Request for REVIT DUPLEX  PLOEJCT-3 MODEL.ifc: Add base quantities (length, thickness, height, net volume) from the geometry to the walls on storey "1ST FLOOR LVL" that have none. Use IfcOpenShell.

First a look at what the model holds.

```python
import ifcopenshell
import ifcopenshell.util.element
import ifcopenshell.util.unit

model = ifcopenshell.open("REVIT DUPLEX  PLOEJCT-3 MODEL.ifc")
print(model.schema)
for unit_type in ("LENGTHUNIT", "AREAUNIT", "VOLUMEUNIT"):
    print(unit_type, ifcopenshell.util.unit.calculate_unit_scale(model, unit_type))
storey = next(s for s in model.by_type("IfcBuildingStorey") if s.Name == "1ST FLOOR LVL")
walls = [e for e in ifcopenshell.util.element.get_decomposition(storey) if e.is_a("IfcWall")]
for e in sorted(walls, key=lambda e: e.id()):
    print(e.id(), e.is_a(), e.Name, list(ifcopenshell.util.element.get_psets(e, qtos_only=True)), sep=" | ")
```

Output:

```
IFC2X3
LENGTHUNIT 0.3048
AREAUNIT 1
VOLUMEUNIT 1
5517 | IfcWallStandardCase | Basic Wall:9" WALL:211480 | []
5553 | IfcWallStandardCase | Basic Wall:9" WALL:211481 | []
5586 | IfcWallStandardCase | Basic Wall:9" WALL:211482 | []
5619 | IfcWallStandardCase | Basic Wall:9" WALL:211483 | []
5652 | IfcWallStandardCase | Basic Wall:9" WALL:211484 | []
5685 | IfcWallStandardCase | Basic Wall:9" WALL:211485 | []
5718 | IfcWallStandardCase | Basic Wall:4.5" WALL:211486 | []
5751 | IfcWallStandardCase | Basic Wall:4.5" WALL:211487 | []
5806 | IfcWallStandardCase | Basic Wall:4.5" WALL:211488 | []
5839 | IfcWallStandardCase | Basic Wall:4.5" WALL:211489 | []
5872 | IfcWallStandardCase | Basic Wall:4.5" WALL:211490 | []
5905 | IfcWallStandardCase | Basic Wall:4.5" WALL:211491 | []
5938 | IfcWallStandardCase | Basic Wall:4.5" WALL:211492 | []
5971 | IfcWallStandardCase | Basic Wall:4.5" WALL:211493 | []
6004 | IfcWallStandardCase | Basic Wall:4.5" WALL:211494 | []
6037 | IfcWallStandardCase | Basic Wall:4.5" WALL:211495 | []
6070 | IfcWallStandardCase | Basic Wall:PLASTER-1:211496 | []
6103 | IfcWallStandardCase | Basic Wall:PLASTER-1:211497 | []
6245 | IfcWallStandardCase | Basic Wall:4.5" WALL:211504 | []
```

```python
import ifcopenshell
import ifcopenshell.api.pset
import ifcopenshell.geom
import ifcopenshell.util.element
import ifcopenshell.util.shape
import ifcopenshell.util.unit

model = ifcopenshell.open("REVIT DUPLEX  PLOEJCT-3 MODEL.ifc")
unit_scale = ifcopenshell.util.unit.calculate_unit_scale(model)
volume_scale = ifcopenshell.util.unit.calculate_unit_scale(model, "VOLUMEUNIT")
settings = ifcopenshell.geom.settings()

storey = next(s for s in model.by_type("IfcBuildingStorey") if s.Name == "1ST FLOOR LVL")
walls = [e for e in ifcopenshell.util.element.get_decomposition(storey) if e.is_a("IfcWall")]

for e in sorted(walls, key=lambda e: e.id()):
    if ifcopenshell.util.element.get_psets(e, qtos_only=True, should_inherit=False):
        continue
    # Geometry comes back in metres, in the element's own axes.
    shape = ifcopenshell.geom.create_shape(settings, e)
    values = {
        "Length": ifcopenshell.util.shape.get_x(shape.geometry) / unit_scale,
        "Width": ifcopenshell.util.shape.get_y(shape.geometry) / unit_scale,
        "Height": ifcopenshell.util.shape.get_z(shape.geometry) / unit_scale,
        "NetVolume": ifcopenshell.util.shape.get_volume(shape.geometry) / volume_scale,
    }
    qto = ifcopenshell.api.pset.add_qto(model, product=e, name="BaseQuantities")
    ifcopenshell.api.pset.edit_qto(model, qto=qto, properties=values)
    print(e.id(), {k: round(v, 3) for k, v in values.items()})

model.write("REVIT DUPLEX  PLOEJCT-3 MODEL_edited.ifc")
```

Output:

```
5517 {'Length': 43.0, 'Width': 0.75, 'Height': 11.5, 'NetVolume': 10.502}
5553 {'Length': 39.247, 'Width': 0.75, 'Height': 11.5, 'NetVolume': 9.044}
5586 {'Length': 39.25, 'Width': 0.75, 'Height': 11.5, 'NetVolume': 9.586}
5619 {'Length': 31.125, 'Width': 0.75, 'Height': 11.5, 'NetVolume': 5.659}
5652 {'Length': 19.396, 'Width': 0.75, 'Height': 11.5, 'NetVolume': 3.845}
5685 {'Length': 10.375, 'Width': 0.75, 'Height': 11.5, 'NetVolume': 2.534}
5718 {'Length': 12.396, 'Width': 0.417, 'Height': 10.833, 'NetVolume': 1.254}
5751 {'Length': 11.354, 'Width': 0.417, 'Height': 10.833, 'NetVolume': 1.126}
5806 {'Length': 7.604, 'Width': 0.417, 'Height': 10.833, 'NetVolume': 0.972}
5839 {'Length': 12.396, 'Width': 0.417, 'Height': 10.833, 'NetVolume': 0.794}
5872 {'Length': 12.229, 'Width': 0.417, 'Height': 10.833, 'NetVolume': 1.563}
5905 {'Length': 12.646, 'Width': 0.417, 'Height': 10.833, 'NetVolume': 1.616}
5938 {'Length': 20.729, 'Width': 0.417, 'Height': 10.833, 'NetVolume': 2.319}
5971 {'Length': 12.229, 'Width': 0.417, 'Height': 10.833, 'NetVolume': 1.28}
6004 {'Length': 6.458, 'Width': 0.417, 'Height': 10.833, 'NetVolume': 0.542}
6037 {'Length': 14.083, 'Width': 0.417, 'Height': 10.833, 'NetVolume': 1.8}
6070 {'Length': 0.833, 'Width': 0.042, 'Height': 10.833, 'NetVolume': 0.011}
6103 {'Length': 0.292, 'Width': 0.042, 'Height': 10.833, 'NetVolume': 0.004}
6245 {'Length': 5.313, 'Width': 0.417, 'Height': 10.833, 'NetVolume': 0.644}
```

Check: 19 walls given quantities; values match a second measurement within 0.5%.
